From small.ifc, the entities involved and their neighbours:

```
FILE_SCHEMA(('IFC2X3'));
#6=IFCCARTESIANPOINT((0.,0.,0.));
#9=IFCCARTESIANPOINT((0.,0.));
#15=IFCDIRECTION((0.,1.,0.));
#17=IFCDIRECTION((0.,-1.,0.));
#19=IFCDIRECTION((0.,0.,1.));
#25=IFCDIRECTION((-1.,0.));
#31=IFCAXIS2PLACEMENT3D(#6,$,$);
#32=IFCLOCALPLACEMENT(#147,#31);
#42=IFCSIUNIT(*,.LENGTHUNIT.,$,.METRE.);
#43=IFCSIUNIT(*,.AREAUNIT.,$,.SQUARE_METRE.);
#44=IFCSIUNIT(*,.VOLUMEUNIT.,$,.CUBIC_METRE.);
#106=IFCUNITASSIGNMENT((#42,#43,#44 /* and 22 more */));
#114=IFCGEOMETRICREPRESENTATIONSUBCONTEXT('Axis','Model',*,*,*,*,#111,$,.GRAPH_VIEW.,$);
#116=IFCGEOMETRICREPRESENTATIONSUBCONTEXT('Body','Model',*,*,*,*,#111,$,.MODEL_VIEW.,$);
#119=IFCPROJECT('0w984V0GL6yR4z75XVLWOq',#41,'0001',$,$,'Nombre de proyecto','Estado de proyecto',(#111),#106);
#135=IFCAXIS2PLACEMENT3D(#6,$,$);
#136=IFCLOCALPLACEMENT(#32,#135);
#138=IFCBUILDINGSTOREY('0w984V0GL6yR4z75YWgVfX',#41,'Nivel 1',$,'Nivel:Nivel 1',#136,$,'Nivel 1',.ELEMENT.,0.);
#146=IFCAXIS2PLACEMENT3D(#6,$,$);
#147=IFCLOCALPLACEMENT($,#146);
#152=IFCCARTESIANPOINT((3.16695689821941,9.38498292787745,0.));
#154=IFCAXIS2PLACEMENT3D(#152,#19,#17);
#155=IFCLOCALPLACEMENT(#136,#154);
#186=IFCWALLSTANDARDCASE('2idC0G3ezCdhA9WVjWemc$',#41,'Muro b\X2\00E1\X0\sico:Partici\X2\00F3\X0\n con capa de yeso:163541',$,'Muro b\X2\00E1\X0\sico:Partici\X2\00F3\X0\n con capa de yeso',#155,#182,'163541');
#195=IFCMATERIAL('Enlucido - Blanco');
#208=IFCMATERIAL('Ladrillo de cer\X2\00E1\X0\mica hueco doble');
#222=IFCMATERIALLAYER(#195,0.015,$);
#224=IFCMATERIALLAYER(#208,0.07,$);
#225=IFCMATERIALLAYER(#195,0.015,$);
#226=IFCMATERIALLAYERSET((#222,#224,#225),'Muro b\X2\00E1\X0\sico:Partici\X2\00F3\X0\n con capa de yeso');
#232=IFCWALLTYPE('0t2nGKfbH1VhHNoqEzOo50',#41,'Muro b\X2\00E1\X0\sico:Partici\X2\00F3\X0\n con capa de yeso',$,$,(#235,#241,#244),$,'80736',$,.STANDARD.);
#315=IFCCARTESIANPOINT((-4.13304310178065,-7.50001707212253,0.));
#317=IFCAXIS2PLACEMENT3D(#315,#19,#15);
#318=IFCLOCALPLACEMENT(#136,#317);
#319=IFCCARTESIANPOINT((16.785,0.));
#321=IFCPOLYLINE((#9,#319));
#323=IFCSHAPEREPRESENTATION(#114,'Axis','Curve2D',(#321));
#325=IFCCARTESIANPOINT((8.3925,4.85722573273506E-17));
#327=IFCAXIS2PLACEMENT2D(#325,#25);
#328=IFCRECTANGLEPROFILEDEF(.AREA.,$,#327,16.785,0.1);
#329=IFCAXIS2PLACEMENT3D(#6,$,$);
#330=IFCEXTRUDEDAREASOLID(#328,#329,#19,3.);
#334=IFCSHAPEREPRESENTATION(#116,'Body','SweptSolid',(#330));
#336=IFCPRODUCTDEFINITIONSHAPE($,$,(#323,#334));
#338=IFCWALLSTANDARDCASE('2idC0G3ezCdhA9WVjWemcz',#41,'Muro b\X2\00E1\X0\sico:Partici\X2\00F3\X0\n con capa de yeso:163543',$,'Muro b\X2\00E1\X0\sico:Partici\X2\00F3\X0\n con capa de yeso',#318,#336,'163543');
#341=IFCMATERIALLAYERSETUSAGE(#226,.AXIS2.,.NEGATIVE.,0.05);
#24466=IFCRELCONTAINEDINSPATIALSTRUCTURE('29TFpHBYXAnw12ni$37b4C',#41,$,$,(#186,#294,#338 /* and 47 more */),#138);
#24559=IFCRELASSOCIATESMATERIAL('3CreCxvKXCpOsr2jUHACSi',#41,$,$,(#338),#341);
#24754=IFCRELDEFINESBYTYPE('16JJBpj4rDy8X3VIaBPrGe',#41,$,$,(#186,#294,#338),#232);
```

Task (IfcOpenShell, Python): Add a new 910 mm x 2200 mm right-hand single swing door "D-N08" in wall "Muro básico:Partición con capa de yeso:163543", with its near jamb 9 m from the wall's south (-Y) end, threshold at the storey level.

```python
import numpy as np
import ifcopenshell
import ifcopenshell.api.feature
import ifcopenshell.api.geometry
import ifcopenshell.api.root
import ifcopenshell.api.spatial
import ifcopenshell.api.type
import ifcopenshell.geom
import ifcopenshell.util.element
import ifcopenshell.util.placement
import ifcopenshell.util.representation
import ifcopenshell.util.shape
import ifcopenshell.util.unit

model = ifcopenshell.open("small.ifc")
unit_scale = ifcopenshell.util.unit.calculate_unit_scale(model)
settings = ifcopenshell.geom.settings()


def volume(element):
    """Net volume in cubic metres, openings subtracted."""
    shape = ifcopenshell.geom.create_shape(settings, element)
    return ifcopenshell.util.shape.get_volume(shape.geometry)


wall = model.by_guid("2idC0G3ezCdhA9WVjWemcz")
storey = ifcopenshell.util.element.get_container(wall, ifc_class="IfcBuildingStorey")
context = ifcopenshell.util.representation.get_context(model, "Model", "Body", "MODEL_VIEW")
before = volume(wall)

width, height, from_end, sill = 0.91, 2.2, 9, 0.0  # metres

# The wall runs along its own X axis, and the end named is its -X end.
wall_shape = ifcopenshell.geom.create_shape(settings, wall)
x, y, z = ifcopenshell.util.shape.get_vertices(wall_shape.geometry).T
start = x.min() + from_end
face, thickness = float(y.min()), float(y.max() - y.min())
wall_matrix = ifcopenshell.util.placement.get_local_placement(wall.ObjectPlacement)
level = ifcopenshell.util.placement.get_local_placement(storey.ObjectPlacement)[2, 3]


def in_wall(x, y):
    """Placement at x, y metres in the wall's axes, at sill height."""
    matrix = wall_matrix.copy()
    matrix[:, 3] = wall_matrix @ np.array([x / unit_scale, y / unit_scale, 0.0, 1.0])
    matrix[2, 3] = level + sill / unit_scale
    return matrix


# Opening: a box that overshoots both wall faces by 50 mm.
opening = ifcopenshell.api.root.create_entity(model, ifc_class="IfcOpeningElement")
box = ifcopenshell.api.geometry.add_wall_representation(
    model, context=context, length=width, height=height, thickness=thickness + 0.1
)
ifcopenshell.api.geometry.assign_representation(model, product=opening, representation=box)
ifcopenshell.api.geometry.edit_object_placement(model, product=opening, matrix=in_wall(start, face - 0.05), is_si=False)
ifcopenshell.api.feature.add_feature(model, feature=opening, element=wall)

door = ifcopenshell.api.root.create_entity(model, ifc_class="IfcDoor", name="D-N08")
door.OverallWidth, door.OverallHeight = width / unit_scale, height / unit_scale
body = ifcopenshell.api.geometry.add_door_representation(
    model,
    context=context,
    overall_width=door.OverallWidth,
    overall_height=door.OverallHeight,
    operation_type="SINGLE_SWING_RIGHT",
    lining_properties={"LiningDepth": thickness / unit_scale, "ThresholdDepth": thickness / unit_scale},
)
ifcopenshell.api.geometry.assign_representation(model, product=door, representation=body)
ifcopenshell.api.spatial.assign_container(model, products=[door], relating_structure=storey)
fills = ifcopenshell.api.feature.add_filling(model, opening=opening, element=door)
fills.OwnerHistory = door.OwnerHistory  # required in IFC2X3

# IFC2X3 keeps the operation on the door style.
style = ifcopenshell.api.root.create_entity(model, ifc_class="IfcDoorStyle", name="D-N08")
style.OperationType, style.ConstructionType = "SINGLE_SWING_RIGHT", "NOTDEFINED"
style.ParameterTakesPrecedence = style.Sizeable = False
ifcopenshell.api.type.assign_type(model, related_objects=[door], relating_type=style)

# The lining spans the wall, so the door starts at the wall face.
ifcopenshell.api.geometry.edit_object_placement(model, product=door, matrix=in_wall(start, face), is_si=False)

after = volume(wall)

print(f"wall volume {before:.3f} -> {after:.3f} m3")

model.write("small_updated.ifc")
```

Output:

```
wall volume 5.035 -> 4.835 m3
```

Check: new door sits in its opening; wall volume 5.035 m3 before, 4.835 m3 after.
